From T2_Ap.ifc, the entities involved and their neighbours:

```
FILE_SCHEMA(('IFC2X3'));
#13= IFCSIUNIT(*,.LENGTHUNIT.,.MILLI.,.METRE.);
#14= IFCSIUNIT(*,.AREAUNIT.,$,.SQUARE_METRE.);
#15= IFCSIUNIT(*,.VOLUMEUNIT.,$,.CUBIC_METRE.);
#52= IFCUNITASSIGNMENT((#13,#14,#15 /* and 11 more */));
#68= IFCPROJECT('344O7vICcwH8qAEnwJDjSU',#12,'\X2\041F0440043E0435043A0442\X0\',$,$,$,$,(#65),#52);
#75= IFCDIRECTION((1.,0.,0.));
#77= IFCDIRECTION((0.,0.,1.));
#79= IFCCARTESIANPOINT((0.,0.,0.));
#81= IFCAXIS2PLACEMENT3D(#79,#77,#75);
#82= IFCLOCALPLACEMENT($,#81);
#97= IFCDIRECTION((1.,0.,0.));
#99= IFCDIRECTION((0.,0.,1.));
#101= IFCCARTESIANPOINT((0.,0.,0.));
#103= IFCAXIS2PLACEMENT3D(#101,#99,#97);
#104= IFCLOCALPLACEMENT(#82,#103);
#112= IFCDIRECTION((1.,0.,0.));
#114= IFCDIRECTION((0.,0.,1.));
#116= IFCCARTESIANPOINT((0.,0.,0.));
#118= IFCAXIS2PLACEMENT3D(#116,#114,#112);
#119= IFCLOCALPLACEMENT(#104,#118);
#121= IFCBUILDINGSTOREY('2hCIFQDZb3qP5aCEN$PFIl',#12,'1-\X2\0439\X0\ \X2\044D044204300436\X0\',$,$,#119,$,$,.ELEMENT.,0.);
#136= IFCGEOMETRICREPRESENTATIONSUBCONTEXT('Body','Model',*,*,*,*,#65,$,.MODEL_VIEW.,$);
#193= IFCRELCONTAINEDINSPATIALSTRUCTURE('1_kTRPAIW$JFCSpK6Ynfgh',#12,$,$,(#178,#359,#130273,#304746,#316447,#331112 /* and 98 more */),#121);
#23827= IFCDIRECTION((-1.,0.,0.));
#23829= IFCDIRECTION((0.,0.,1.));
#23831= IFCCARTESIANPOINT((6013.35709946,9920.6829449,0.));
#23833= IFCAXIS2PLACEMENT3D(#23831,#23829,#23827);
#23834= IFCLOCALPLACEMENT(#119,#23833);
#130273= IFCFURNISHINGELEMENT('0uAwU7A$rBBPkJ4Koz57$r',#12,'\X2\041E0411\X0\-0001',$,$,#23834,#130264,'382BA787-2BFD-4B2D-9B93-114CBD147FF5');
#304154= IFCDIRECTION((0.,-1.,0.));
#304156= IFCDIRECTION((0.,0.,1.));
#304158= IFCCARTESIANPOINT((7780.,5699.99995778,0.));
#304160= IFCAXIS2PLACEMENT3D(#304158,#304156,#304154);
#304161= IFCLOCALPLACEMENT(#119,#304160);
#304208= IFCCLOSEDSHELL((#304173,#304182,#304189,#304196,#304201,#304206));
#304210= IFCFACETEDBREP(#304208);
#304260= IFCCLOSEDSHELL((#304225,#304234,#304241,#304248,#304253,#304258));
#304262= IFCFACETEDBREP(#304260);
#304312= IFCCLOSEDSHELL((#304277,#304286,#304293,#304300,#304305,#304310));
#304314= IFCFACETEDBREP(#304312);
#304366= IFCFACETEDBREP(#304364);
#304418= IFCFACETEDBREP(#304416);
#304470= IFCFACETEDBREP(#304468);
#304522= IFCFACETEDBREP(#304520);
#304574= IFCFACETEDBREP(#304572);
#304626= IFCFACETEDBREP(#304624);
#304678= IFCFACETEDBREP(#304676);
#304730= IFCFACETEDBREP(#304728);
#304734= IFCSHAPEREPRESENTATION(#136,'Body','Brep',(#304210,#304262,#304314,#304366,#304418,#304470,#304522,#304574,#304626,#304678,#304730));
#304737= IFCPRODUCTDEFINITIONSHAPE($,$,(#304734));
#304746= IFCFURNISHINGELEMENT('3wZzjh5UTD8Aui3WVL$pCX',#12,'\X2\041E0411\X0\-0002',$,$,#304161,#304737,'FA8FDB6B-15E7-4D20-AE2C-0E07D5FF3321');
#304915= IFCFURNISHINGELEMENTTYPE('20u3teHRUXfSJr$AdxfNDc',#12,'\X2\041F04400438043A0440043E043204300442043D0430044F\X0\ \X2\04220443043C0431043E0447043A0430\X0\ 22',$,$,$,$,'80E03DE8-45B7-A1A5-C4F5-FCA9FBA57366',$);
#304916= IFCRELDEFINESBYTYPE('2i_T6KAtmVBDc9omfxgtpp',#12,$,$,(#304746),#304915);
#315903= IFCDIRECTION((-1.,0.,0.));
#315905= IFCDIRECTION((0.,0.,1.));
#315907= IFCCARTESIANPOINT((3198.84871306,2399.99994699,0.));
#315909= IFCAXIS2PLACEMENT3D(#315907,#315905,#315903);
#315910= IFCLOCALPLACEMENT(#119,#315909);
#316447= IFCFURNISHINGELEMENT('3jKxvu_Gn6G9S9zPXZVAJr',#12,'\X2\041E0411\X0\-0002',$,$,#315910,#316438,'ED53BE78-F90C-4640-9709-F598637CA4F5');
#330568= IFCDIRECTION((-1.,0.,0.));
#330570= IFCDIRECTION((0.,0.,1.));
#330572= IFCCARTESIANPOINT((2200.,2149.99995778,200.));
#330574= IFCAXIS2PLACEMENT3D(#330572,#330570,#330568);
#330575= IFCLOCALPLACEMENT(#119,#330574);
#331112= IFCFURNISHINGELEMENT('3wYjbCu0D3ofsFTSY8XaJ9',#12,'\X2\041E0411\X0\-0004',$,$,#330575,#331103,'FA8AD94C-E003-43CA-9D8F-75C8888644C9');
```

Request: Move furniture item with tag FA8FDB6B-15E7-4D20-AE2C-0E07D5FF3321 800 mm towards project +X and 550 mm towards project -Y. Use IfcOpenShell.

```python
import ifcopenshell
import ifcopenshell.api.geometry
import ifcopenshell.util.placement
import ifcopenshell.util.unit

model = ifcopenshell.open("T2_Ap.ifc")
unit_scale = ifcopenshell.util.unit.calculate_unit_scale(model)

item = model.by_id(304746)
matrix = ifcopenshell.util.placement.get_local_placement(item.ObjectPlacement)
matrix[0, 3] += 0.8 / unit_scale
matrix[1, 3] -= 0.55 / unit_scale
ifcopenshell.api.geometry.edit_object_placement(model, product=item, matrix=matrix, is_si=False)

print(ifcopenshell.util.placement.get_local_placement(item.ObjectPlacement).round(3) + 0.0)

model.write("T2_Ap-out.ifc")
```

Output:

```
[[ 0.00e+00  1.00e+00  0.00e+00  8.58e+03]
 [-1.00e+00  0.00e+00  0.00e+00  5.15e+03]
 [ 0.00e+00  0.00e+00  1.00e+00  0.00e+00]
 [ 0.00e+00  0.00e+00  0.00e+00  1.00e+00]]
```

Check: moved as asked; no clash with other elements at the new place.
